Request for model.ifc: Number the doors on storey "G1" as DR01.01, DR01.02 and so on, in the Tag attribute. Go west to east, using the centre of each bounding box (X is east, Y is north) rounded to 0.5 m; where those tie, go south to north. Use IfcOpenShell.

First a look at what the model holds.

```python
import ifcopenshell
import ifcopenshell.util.element
import ifcopenshell.util.placement

model = ifcopenshell.open("model.ifc")
print(model.schema)
storey = next(s for s in model.by_type("IfcBuildingStorey") if s.Name == "G1")
doors = [e for e in ifcopenshell.util.element.get_decomposition(storey) if e.is_a("IfcDoor")]
for e in sorted(doors, key=lambda e: e.id()):
    origin = ifcopenshell.util.placement.get_local_placement(e.ObjectPlacement)[:3, 3]
    print(e.id(), e.Tag, e.Name, origin.round(2) + 0.0, sep=" | ")
```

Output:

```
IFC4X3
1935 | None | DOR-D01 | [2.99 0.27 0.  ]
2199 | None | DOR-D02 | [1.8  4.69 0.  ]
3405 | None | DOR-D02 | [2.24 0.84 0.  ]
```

```python
import ifcopenshell
import ifcopenshell.geom
import ifcopenshell.util.element
import ifcopenshell.util.shape

model = ifcopenshell.open("model.ifc")
settings = ifcopenshell.geom.settings()
settings.set("use-world-coords", True)


def centre(element):
    shape = ifcopenshell.geom.create_shape(settings, element)
    return ifcopenshell.util.shape.get_bbox_centroid(shape.geometry)


storey = next(s for s in model.by_type("IfcBuildingStorey") if s.Name == "G1")
doors = [e for e in ifcopenshell.util.element.get_decomposition(storey) if e.is_a("IfcDoor")]

# Insertion points can sit at a corner or the storey origin, so sort by the geometry (in metres).
centres = {e: centre(e) for e in doors}
doors.sort(key=lambda e: (round(centres[e][0] / 0.5), centres[e][1]))

for i, e in enumerate(doors, start=1):
    number = f"DR01.{i:02d}"
    e.Tag = number
    print(e.id(), number)

model.write("model_updated.ifc")
```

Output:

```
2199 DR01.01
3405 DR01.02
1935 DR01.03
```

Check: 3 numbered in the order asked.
